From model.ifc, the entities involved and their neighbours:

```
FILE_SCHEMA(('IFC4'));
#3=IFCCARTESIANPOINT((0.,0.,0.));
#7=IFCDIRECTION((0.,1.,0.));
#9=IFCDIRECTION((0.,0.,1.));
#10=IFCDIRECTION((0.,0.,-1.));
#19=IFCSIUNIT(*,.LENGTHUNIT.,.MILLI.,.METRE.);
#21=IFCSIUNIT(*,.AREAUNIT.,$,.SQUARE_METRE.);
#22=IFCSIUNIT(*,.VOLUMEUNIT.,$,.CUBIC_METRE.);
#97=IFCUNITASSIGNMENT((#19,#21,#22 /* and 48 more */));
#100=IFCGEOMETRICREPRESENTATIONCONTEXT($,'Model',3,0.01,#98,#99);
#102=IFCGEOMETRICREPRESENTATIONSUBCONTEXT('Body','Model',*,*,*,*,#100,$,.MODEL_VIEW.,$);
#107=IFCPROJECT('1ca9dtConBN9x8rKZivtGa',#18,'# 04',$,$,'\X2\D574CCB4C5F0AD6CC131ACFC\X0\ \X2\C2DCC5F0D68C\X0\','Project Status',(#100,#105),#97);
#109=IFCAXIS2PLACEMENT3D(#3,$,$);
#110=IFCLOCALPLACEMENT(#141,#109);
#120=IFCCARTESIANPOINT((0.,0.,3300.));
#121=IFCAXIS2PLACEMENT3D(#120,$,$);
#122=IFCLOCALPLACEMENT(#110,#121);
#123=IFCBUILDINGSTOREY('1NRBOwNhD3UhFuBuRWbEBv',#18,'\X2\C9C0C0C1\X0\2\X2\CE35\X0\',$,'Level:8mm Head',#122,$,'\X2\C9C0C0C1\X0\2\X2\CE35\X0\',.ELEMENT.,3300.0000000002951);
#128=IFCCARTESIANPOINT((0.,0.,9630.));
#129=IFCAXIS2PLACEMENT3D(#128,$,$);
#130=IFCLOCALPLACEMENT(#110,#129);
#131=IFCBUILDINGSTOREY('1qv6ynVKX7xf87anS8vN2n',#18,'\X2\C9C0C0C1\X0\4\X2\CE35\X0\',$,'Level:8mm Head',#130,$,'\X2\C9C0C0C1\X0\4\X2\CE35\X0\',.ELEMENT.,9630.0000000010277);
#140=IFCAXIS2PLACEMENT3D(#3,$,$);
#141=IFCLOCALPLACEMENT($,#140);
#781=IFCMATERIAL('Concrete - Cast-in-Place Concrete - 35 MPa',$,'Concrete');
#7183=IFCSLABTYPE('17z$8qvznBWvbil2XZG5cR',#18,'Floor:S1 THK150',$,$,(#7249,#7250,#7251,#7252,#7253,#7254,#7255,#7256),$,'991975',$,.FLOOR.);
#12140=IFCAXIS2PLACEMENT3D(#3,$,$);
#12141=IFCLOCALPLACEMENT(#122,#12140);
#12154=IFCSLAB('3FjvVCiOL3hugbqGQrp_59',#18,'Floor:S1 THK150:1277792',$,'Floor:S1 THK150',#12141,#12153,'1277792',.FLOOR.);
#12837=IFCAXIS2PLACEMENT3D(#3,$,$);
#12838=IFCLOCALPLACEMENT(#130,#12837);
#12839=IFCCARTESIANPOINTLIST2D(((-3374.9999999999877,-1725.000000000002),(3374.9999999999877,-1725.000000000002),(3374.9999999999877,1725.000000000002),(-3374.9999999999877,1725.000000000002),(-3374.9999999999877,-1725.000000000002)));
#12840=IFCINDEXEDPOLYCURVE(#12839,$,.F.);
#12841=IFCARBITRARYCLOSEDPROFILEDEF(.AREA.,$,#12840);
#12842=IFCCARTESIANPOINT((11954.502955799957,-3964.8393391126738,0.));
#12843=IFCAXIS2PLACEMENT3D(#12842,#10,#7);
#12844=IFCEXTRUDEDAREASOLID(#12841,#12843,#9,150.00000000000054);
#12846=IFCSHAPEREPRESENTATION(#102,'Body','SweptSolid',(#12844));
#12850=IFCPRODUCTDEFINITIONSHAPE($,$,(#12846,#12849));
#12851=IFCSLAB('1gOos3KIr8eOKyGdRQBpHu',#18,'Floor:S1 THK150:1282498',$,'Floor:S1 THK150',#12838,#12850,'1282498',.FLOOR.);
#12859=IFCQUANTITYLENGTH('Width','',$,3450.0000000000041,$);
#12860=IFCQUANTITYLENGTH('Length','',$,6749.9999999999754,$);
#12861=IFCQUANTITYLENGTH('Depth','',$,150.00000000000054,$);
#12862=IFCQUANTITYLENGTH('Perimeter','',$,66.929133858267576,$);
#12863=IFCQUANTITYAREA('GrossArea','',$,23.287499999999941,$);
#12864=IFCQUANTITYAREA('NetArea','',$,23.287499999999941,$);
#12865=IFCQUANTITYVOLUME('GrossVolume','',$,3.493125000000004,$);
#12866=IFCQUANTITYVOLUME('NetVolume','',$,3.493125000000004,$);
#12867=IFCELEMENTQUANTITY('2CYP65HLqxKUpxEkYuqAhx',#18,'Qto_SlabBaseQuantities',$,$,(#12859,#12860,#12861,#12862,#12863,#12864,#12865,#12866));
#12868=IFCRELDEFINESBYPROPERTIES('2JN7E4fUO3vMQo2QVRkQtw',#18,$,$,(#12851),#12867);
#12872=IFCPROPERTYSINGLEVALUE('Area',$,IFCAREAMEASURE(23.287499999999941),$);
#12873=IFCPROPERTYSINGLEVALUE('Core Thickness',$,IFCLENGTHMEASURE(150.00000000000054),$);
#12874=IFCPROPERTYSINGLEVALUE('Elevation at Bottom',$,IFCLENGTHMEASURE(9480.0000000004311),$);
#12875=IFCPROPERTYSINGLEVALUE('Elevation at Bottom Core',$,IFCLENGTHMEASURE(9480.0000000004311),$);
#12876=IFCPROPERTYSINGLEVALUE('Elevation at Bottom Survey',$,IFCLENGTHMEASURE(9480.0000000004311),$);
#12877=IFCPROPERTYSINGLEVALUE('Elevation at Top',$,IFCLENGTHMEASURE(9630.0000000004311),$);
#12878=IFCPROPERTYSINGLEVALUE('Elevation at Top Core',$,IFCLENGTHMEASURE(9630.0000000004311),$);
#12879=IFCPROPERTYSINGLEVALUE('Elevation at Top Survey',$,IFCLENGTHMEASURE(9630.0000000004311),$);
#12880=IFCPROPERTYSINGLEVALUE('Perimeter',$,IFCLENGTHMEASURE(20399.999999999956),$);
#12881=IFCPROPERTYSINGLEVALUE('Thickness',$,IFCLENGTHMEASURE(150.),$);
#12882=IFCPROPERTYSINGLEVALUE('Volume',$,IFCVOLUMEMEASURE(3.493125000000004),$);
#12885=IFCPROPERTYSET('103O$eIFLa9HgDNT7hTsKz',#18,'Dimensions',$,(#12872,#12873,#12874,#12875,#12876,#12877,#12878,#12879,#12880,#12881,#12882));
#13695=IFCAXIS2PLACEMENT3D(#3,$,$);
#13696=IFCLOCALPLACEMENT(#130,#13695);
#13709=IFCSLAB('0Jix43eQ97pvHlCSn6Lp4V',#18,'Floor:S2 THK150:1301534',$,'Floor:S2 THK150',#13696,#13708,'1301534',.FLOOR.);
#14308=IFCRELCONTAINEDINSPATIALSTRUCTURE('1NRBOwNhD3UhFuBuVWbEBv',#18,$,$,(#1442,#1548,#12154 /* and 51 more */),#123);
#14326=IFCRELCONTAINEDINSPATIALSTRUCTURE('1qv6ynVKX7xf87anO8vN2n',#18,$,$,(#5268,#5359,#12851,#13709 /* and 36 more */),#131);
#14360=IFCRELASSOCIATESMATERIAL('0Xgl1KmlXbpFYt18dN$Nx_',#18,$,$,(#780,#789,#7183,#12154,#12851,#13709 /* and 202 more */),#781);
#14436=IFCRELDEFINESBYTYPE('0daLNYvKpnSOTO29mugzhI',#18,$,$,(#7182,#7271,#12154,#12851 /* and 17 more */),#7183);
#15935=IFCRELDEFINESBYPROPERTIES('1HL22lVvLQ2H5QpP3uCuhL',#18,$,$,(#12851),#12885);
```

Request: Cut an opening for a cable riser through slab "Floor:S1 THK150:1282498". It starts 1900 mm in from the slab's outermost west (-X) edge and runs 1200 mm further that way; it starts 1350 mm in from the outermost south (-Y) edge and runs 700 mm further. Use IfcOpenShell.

```python
import numpy as np
import ifcopenshell
import ifcopenshell.api.feature
import ifcopenshell.api.geometry
import ifcopenshell.api.pset
import ifcopenshell.api.root
import ifcopenshell.geom
import ifcopenshell.util.element
import ifcopenshell.util.placement
import ifcopenshell.util.representation
import ifcopenshell.util.shape
import ifcopenshell.util.unit

model = ifcopenshell.open("model.ifc")
unit_scale = ifcopenshell.util.unit.calculate_unit_scale(model)
area_scale = ifcopenshell.util.unit.calculate_unit_scale(model, "AREAUNIT")
volume_scale = ifcopenshell.util.unit.calculate_unit_scale(model, "VOLUMEUNIT")
settings = ifcopenshell.geom.settings()


def volume(element):
    """Net volume in cubic metres, openings subtracted."""
    shape = ifcopenshell.geom.create_shape(settings, element)
    return ifcopenshell.util.shape.get_volume(shape.geometry)


slab = model.by_guid("1gOos3KIr8eOKyGdRQBpHu")
before = volume(slab)

# Extent in the slab's own axes, in metres. The edges named are its -X and -Y sides.
slab_shape = ifcopenshell.geom.create_shape(settings, slab)
vertices = ifcopenshell.util.shape.get_vertices(slab_shape.geometry)
x_min, y_min, bottom = vertices.min(axis=0)
top = vertices[:, 2].max()

opening = ifcopenshell.api.root.create_entity(model, ifc_class="IfcOpeningElement", name="Cable riser opening", predefined_type="OPENING")
context = ifcopenshell.util.representation.get_context(model, "Model", "Body", "MODEL_VIEW")
width, depth = 1.2, 0.7
outline = [(0.0, 0.0), (width, 0.0), (width, depth), (0.0, depth), (0.0, 0.0)]
# Overshoot both faces by 50 mm so the cut is clean.
shape = ifcopenshell.api.geometry.add_slab_representation(
    model, context=context, depth=top - bottom + 0.1, polyline=outline
)
ifcopenshell.api.geometry.assign_representation(model, product=opening, representation=shape)

matrix = ifcopenshell.util.placement.get_local_placement(slab.ObjectPlacement)
matrix[:, 3] = matrix @ np.append(np.array([x_min + 1.9, y_min + 1.35, bottom - 0.05]) / unit_scale, 1.0)
ifcopenshell.api.geometry.edit_object_placement(model, product=opening, matrix=matrix, is_si=False)
ifcopenshell.api.feature.add_feature(model, feature=opening, element=slab)

after = volume(slab)

# Update the slab's stored quantities.
qto = model.by_id(ifcopenshell.util.element.get_pset(slab, "Qto_SlabBaseQuantities", should_inherit=False)["id"])
ifcopenshell.api.pset.edit_qto(model, qto=qto, properties={
    "NetArea": after / (top - bottom) / area_scale,
    "NetVolume": after / volume_scale,
})
pset = model.by_id(ifcopenshell.util.element.get_pset(slab, "Dimensions", should_inherit=False)["id"])
ifcopenshell.api.pset.edit_pset(model, pset=pset, properties={
    "Area": model.create_entity("IfcAreaMeasure", after / (top - bottom) / area_scale),
    "Volume": model.create_entity("IfcVolumeMeasure", after / volume_scale),
})

print(f"slab volume {before:.3f} -> {after:.3f} m3")

model.write("model_edited.ifc")
```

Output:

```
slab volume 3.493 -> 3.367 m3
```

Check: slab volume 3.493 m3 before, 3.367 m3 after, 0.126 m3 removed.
